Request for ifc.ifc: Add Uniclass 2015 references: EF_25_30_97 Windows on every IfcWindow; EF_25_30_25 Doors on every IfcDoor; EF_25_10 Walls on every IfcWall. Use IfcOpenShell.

First a look at what the model holds.

```python
import ifcopenshell

model = ifcopenshell.open("ifc.ifc")
print(model.schema)
print("classifications:", [c.Name for c in model.by_type("IfcClassification")])
for ifc_class in ("IfcDoor", "IfcRoof", "IfcStair", "IfcWall", "IfcWindow"):
    print(ifc_class, len(model.by_type(ifc_class)))
```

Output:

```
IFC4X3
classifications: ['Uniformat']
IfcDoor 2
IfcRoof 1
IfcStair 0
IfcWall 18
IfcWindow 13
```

```python
import ifcopenshell
import ifcopenshell.api.classification

model = ifcopenshell.open("ifc.ifc")

system = ifcopenshell.api.classification.add_classification(model, classification="Uniclass 2015")

codes = {
    "IfcWindow": ("EF_25_30_97", "Windows"),
    "IfcDoor": ("EF_25_30_25", "Doors"),
    "IfcWall": ("EF_25_10", "Walls"),
}
for ifc_class, (code, name) in codes.items():
    products = model.by_type(ifc_class)
    ifcopenshell.api.classification.add_reference(
        model, products=products, classification=system, identification=code, name=name
    )
    print(code, len(products))

model.write("ifc_rev.ifc")
```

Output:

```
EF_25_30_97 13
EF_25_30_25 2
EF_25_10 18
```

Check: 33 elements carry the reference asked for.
